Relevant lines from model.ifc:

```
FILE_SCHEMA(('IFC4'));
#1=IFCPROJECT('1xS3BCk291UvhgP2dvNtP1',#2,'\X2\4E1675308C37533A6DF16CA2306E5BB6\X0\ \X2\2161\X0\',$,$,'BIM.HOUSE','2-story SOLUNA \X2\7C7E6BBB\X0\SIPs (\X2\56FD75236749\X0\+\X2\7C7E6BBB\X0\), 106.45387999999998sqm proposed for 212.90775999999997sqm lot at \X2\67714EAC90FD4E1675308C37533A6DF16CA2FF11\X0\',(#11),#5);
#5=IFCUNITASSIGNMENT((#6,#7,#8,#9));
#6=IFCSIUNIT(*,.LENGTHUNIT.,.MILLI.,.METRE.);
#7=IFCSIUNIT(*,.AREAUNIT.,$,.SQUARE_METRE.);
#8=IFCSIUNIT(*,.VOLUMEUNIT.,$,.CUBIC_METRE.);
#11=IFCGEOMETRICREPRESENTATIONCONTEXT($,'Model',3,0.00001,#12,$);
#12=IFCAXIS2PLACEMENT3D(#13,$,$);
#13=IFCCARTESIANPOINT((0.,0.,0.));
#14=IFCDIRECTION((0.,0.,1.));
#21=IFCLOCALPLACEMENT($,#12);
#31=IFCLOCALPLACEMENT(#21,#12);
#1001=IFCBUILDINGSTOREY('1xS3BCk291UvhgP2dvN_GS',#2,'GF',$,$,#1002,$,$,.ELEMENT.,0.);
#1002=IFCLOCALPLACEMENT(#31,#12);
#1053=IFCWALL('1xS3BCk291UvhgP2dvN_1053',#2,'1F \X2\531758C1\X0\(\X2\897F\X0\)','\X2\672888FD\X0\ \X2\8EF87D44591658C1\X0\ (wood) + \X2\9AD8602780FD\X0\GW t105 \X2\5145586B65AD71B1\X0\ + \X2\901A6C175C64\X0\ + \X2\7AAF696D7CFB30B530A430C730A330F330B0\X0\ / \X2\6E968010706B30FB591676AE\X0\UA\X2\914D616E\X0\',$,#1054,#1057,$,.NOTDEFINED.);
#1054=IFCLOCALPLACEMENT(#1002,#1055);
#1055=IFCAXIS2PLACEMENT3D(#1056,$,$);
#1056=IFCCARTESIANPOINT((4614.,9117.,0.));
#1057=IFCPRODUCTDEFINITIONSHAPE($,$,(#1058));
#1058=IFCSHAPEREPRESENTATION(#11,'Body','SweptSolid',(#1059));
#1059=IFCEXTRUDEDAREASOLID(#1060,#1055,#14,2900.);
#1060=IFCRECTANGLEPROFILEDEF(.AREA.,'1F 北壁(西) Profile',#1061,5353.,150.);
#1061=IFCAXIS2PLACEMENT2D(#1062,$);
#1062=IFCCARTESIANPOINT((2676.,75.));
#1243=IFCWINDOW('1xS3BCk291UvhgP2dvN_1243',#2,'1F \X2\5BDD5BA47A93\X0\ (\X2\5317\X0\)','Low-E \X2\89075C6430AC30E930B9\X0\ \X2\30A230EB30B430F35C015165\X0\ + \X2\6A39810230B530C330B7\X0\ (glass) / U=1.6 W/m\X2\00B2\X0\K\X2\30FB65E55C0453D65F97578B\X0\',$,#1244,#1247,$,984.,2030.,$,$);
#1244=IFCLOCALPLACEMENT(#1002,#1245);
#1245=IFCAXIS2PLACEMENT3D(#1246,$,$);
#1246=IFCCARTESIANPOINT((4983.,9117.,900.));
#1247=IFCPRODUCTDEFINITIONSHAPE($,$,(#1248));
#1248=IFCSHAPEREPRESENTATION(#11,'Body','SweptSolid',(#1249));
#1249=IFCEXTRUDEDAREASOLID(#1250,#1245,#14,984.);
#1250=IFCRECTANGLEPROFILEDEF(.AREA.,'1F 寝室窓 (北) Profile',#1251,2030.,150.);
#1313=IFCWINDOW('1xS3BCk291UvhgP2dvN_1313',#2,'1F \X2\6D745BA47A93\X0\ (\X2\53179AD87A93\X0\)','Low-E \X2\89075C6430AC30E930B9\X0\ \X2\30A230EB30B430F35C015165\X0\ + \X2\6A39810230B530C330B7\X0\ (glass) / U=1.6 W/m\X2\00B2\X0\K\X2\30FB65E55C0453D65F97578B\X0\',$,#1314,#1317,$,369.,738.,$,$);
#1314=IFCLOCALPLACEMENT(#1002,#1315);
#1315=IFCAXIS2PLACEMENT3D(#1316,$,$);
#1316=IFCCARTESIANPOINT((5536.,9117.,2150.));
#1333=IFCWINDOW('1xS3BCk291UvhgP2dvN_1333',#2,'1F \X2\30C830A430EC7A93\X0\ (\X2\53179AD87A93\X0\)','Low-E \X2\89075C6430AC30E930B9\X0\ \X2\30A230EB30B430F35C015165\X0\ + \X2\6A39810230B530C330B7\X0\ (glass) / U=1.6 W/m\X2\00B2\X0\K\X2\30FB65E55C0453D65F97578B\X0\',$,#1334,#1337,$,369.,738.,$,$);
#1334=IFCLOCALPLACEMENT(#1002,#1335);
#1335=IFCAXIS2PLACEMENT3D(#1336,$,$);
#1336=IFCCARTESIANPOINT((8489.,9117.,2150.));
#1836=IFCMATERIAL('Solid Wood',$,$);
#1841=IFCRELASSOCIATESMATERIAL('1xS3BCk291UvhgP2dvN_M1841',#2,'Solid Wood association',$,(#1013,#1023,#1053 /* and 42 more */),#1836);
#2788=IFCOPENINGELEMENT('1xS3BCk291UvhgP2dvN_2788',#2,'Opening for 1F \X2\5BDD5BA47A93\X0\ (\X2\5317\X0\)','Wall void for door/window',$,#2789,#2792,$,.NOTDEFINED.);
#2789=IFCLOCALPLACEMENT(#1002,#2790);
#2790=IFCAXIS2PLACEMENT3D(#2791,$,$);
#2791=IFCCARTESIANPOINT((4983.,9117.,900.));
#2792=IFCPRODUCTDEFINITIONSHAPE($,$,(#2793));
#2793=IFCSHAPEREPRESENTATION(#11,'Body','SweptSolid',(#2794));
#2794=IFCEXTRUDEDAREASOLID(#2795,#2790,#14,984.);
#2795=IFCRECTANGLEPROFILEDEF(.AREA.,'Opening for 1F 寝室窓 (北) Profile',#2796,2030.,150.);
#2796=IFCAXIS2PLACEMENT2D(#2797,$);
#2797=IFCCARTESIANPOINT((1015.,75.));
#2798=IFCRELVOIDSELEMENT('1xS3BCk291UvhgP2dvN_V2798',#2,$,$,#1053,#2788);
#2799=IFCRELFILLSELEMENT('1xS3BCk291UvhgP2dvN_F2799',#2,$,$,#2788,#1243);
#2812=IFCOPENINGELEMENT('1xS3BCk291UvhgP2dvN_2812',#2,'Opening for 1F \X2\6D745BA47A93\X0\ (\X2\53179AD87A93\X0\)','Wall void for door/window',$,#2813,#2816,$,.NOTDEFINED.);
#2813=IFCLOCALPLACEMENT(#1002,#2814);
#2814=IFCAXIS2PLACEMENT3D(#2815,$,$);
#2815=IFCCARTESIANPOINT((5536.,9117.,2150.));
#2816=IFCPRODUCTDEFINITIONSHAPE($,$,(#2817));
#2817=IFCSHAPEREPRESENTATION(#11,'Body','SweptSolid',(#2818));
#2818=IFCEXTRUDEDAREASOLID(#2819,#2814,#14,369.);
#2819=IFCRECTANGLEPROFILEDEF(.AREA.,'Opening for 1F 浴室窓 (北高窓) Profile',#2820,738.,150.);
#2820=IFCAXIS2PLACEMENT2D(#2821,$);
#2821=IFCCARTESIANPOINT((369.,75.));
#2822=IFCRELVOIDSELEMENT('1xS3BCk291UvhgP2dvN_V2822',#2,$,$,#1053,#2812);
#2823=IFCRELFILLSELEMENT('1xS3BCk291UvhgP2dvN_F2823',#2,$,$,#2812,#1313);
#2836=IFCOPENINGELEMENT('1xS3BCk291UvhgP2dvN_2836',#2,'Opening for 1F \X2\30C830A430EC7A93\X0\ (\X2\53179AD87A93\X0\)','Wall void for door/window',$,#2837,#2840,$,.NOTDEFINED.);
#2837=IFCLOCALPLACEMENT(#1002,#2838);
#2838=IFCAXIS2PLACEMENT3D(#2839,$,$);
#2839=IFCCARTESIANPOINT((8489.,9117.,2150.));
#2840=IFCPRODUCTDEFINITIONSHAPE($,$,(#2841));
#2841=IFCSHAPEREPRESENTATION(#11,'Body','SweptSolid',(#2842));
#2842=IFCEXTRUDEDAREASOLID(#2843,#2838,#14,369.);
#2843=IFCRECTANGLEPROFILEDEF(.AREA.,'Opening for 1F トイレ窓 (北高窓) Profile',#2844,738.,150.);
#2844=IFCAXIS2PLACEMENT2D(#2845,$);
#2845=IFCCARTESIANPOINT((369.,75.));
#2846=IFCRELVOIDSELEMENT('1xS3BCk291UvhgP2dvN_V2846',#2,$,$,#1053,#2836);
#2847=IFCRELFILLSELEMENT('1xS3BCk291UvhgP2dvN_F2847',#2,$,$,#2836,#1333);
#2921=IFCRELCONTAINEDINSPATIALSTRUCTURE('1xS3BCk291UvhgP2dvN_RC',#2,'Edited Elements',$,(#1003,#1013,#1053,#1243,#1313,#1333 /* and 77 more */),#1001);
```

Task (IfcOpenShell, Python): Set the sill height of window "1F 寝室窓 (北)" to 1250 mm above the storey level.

```python
import numpy as np
import ifcopenshell
import ifcopenshell.api.geometry
import ifcopenshell.geom
import ifcopenshell.util.element
import ifcopenshell.util.placement
import ifcopenshell.util.shape
import ifcopenshell.util.unit

model = ifcopenshell.open("model.ifc")
unit_scale = ifcopenshell.util.unit.calculate_unit_scale(model)

window = model.by_id(1243)
opening = window.FillsVoids[0].RelatingOpeningElement
storey = ifcopenshell.util.element.get_container(window, ifc_class="IfcBuildingStorey")
level = ifcopenshell.util.placement.get_local_placement(storey.ObjectPlacement)[2, 3]

# The opening's origin need not be at the sill, so measure its lowest point.
shape = ifcopenshell.geom.create_shape(ifcopenshell.geom.settings(), opening)
bottom = ifcopenshell.util.shape.get_shape_bottom_elevation(shape, shape.geometry) / unit_scale
dz = level + 1.25 / unit_scale - bottom

shift = np.array([0.0, 0.0, dz])
# The window is not placed relative to its opening, so move both.
for product in (opening, window):
    matrix = ifcopenshell.util.placement.get_local_placement(product.ObjectPlacement)
    matrix[:3, 3] += shift
    ifcopenshell.api.geometry.edit_object_placement(model, product=product, matrix=matrix, is_si=False)

print(f"moved by {dz * unit_scale:+.3f} m")

model.write("model_updated.ifc")
```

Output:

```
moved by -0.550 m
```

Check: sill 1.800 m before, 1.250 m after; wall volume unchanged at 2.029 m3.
